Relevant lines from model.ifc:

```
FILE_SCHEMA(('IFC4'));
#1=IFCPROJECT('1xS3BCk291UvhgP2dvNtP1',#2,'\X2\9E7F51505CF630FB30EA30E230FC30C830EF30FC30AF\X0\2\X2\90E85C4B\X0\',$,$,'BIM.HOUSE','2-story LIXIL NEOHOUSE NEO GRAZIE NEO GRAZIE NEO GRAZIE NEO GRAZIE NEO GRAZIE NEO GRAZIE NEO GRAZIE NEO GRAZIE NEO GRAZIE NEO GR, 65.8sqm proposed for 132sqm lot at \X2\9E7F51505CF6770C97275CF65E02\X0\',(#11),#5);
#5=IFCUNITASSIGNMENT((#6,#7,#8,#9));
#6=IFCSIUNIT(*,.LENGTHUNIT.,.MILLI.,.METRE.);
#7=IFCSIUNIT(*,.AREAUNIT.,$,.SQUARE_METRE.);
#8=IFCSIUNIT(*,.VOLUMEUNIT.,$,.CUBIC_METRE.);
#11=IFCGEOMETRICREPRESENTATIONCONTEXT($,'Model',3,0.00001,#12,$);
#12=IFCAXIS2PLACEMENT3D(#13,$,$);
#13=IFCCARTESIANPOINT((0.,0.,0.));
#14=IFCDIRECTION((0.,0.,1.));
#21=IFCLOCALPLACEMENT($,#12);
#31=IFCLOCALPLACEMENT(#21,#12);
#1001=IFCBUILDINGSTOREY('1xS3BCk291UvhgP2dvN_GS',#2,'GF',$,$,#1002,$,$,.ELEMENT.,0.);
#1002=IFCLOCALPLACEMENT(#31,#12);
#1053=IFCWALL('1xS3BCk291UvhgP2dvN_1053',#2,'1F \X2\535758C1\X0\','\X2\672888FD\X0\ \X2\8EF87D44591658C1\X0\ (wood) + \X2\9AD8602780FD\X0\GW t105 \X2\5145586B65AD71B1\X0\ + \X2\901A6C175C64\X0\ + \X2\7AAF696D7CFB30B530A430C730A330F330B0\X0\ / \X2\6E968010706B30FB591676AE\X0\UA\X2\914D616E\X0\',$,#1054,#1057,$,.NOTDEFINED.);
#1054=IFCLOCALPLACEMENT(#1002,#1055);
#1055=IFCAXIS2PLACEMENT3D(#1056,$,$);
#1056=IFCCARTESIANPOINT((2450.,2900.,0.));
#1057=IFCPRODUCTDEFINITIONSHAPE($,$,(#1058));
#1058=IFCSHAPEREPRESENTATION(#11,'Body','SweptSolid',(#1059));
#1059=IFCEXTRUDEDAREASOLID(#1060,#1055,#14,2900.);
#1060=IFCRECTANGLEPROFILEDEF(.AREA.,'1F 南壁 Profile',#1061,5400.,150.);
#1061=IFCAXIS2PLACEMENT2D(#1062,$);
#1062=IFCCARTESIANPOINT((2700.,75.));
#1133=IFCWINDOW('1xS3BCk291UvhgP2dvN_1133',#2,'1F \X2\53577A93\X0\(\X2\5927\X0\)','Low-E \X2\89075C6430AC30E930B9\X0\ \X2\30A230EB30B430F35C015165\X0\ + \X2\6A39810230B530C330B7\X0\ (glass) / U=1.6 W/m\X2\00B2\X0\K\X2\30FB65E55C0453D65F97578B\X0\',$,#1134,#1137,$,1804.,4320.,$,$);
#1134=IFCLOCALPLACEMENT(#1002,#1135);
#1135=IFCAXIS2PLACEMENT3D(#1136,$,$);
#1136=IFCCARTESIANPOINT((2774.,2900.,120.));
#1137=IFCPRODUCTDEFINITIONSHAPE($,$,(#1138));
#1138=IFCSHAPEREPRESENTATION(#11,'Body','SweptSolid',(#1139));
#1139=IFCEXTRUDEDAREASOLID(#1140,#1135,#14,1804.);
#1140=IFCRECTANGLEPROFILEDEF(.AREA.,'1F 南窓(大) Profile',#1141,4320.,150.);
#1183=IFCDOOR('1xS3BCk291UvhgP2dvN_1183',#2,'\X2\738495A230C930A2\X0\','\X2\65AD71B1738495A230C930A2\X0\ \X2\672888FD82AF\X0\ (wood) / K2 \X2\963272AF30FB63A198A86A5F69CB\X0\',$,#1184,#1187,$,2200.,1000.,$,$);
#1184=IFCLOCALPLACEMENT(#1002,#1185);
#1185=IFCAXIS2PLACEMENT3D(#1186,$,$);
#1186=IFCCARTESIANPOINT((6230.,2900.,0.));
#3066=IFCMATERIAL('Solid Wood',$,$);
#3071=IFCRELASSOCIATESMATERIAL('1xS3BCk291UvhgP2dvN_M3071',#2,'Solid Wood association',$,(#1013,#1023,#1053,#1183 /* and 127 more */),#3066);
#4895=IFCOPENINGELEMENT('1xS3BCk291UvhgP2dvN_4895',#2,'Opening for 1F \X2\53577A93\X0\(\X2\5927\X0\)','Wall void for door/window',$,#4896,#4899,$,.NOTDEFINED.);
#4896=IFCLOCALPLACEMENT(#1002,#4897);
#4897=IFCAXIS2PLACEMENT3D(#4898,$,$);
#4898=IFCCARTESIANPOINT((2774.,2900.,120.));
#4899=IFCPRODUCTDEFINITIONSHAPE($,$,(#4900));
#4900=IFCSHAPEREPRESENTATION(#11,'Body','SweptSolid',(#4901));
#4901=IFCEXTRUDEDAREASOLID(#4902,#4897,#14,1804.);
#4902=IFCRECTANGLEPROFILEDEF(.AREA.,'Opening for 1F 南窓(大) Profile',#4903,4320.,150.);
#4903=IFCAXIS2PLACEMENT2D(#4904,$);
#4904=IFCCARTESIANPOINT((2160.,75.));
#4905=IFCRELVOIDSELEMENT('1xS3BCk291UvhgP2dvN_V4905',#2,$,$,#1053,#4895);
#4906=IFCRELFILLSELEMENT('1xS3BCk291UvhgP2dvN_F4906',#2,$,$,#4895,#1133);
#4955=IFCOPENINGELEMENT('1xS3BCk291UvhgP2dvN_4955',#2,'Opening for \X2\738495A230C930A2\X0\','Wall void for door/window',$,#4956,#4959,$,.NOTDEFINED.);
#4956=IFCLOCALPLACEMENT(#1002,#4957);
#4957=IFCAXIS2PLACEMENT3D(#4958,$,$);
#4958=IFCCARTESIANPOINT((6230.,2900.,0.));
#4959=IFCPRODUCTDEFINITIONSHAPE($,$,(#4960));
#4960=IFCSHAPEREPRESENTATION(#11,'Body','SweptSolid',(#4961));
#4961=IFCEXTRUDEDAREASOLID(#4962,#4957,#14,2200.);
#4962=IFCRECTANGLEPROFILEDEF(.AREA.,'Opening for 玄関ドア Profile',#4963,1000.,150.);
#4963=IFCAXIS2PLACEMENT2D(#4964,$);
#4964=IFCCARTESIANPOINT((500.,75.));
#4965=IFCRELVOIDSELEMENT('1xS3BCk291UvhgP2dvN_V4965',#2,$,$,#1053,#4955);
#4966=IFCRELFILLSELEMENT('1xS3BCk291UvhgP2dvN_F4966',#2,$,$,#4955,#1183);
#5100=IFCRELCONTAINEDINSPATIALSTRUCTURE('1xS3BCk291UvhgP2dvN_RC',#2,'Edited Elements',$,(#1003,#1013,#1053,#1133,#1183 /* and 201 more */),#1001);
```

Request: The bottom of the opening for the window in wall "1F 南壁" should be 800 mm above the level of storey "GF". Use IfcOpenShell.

```python
import numpy as np
import ifcopenshell
import ifcopenshell.api.geometry
import ifcopenshell.geom
import ifcopenshell.util.element
import ifcopenshell.util.placement
import ifcopenshell.util.shape
import ifcopenshell.util.unit

model = ifcopenshell.open("model.ifc")
unit_scale = ifcopenshell.util.unit.calculate_unit_scale(model)

window = model.by_guid("1xS3BCk291UvhgP2dvN_1133")
opening = window.FillsVoids[0].RelatingOpeningElement
storey = ifcopenshell.util.element.get_container(window, ifc_class="IfcBuildingStorey")
level = ifcopenshell.util.placement.get_local_placement(storey.ObjectPlacement)[2, 3]

# The opening's origin need not be at the sill, so measure its lowest point.
shape = ifcopenshell.geom.create_shape(ifcopenshell.geom.settings(), opening)
bottom = ifcopenshell.util.shape.get_shape_bottom_elevation(shape, shape.geometry) / unit_scale
dz = level + 800.0 - bottom

shift = np.array([0.0, 0.0, dz])
# The window is not placed relative to its opening, so move both.
for product in (opening, window):
    matrix = ifcopenshell.util.placement.get_local_placement(product.ObjectPlacement)
    matrix[:3, 3] += shift
    ifcopenshell.api.geometry.edit_object_placement(model, product=product, matrix=matrix, is_si=False)

print(f"moved by {dz * unit_scale:+.3f} m")

model.write("model_rev.ifc")
```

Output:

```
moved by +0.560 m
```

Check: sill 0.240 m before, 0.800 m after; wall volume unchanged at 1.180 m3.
